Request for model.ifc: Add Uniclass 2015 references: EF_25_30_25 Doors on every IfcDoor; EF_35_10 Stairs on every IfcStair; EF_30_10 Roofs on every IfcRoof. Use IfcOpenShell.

First a look at what the model holds.

```python
import ifcopenshell

model = ifcopenshell.open("model.ifc")
print(model.schema)
print("classifications:", [c.Name for c in model.by_type("IfcClassification")])
for ifc_class in ("IfcDoor", "IfcRoof", "IfcStair", "IfcWall", "IfcWindow"):
    print(ifc_class, len(model.by_type(ifc_class)))
```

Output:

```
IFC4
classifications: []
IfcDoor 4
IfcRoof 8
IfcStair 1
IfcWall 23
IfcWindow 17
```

```python
import ifcopenshell
import ifcopenshell.api.classification

model = ifcopenshell.open("model.ifc")

system = ifcopenshell.api.classification.add_classification(model, classification="Uniclass 2015")

codes = {
    "IfcDoor": ("EF_25_30_25", "Doors"),
    "IfcStair": ("EF_35_10", "Stairs"),
    "IfcRoof": ("EF_30_10", "Roofs"),
}
for ifc_class, (code, name) in codes.items():
    products = model.by_type(ifc_class)
    ifcopenshell.api.classification.add_reference(
        model, products=products, classification=system, identification=code, name=name
    )
    print(code, len(products))

model.write("model_rev.ifc")
```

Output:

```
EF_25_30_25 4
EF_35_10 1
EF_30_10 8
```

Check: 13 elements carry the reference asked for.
